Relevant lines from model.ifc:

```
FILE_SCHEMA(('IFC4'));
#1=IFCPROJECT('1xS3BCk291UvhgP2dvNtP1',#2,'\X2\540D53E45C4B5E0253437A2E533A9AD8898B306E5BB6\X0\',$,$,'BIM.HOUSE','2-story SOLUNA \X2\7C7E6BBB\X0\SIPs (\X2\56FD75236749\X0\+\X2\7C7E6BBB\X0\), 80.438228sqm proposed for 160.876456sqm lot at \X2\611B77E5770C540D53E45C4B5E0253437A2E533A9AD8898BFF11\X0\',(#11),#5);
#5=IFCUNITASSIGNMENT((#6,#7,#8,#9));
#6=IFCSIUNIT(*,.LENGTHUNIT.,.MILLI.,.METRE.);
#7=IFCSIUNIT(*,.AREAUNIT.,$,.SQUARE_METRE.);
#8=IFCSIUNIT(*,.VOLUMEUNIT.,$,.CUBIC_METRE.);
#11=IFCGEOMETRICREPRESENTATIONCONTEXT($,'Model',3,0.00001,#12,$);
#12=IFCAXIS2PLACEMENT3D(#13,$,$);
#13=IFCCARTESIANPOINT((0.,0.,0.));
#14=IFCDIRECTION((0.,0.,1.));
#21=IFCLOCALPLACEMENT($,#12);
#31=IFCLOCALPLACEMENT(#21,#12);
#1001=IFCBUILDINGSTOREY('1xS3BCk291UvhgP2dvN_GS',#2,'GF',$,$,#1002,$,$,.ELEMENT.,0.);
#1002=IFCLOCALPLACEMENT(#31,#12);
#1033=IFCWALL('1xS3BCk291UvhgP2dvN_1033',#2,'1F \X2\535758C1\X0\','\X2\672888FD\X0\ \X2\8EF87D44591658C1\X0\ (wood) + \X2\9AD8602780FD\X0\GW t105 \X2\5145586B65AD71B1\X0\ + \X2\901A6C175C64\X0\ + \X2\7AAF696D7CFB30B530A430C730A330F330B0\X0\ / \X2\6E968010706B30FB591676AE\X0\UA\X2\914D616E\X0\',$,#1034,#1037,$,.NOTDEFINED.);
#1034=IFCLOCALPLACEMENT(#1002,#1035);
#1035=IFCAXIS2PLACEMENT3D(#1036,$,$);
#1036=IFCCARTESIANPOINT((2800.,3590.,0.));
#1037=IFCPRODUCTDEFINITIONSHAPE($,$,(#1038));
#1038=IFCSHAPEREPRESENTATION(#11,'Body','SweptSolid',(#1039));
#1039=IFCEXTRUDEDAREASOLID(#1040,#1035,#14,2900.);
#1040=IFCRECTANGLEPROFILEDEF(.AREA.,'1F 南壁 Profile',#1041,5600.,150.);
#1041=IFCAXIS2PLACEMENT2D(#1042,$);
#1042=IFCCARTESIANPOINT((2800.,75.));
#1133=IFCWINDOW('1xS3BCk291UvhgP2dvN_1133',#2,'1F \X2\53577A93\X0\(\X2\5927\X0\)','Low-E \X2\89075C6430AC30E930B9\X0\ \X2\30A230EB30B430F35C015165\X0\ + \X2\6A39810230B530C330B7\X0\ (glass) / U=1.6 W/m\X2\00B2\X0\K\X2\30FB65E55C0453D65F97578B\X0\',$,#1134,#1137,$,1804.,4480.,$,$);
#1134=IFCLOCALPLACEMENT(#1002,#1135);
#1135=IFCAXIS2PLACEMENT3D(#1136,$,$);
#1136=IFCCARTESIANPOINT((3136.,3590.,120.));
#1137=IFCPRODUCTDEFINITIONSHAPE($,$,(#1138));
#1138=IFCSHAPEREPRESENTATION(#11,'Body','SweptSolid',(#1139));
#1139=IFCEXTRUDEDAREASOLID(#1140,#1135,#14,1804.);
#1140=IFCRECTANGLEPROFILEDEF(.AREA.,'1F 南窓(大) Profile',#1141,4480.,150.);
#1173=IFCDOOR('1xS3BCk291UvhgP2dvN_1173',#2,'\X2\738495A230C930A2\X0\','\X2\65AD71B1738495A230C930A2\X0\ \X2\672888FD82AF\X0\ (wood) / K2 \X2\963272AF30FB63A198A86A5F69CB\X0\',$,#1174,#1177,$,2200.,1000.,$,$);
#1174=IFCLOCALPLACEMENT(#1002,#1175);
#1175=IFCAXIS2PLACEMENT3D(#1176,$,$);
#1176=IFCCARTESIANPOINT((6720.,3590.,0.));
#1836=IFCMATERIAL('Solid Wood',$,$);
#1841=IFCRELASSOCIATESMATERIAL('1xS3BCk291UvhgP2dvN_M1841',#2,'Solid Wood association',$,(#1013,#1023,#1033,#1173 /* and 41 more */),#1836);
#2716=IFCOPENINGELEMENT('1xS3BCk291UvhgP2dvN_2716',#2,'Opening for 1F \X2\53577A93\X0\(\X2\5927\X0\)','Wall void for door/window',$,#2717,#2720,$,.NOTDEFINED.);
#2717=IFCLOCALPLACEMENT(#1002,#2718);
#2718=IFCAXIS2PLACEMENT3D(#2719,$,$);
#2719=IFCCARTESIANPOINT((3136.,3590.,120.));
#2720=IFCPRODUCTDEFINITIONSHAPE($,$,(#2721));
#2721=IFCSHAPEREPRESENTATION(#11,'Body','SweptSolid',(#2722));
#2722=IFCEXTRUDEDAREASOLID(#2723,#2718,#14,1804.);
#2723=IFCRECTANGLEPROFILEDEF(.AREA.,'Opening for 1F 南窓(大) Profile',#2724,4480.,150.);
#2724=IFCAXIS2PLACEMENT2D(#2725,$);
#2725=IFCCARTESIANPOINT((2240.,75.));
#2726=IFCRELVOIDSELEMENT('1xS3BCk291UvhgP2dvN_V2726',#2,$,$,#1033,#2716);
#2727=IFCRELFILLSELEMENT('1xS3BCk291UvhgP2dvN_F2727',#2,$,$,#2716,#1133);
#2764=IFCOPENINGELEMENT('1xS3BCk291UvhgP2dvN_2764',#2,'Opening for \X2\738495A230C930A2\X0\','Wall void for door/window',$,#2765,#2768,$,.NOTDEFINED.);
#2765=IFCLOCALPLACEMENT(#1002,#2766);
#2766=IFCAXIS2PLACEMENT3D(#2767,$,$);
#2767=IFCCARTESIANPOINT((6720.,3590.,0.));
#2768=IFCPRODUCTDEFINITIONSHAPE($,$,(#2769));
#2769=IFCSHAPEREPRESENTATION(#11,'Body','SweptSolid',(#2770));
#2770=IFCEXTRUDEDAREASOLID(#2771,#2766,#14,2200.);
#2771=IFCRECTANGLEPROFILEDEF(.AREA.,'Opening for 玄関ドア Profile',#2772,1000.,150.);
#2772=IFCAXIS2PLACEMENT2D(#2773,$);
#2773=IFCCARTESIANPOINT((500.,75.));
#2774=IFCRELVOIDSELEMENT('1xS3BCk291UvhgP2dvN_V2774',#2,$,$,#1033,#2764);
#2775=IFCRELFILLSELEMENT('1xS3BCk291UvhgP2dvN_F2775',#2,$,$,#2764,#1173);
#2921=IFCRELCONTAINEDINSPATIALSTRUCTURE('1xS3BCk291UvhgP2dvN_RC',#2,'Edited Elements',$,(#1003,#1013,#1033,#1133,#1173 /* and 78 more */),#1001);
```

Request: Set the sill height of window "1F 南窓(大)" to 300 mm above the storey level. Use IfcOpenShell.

```python
import numpy as np
import ifcopenshell
import ifcopenshell.api.geometry
import ifcopenshell.geom
import ifcopenshell.util.element
import ifcopenshell.util.placement
import ifcopenshell.util.shape
import ifcopenshell.util.unit

model = ifcopenshell.open("model.ifc")
unit_scale = ifcopenshell.util.unit.calculate_unit_scale(model)

window = model.by_guid("1xS3BCk291UvhgP2dvN_1133")
opening = window.FillsVoids[0].RelatingOpeningElement
storey = ifcopenshell.util.element.get_container(window, ifc_class="IfcBuildingStorey")
level = ifcopenshell.util.placement.get_local_placement(storey.ObjectPlacement)[2, 3]

# The opening's origin need not be at the sill, so measure its lowest point.
shape = ifcopenshell.geom.create_shape(ifcopenshell.geom.settings(), opening)
bottom = ifcopenshell.util.shape.get_shape_bottom_elevation(shape, shape.geometry) / unit_scale
dz = level + 0.3 / unit_scale - bottom

shift = np.array([0.0, 0.0, dz])
# The window is not placed relative to its opening, so move both.
for product in (opening, window):
    matrix = ifcopenshell.util.placement.get_local_placement(product.ObjectPlacement)
    matrix[:3, 3] += shift
    ifcopenshell.api.geometry.edit_object_placement(model, product=product, matrix=matrix, is_si=False)

print(f"moved by {dz * unit_scale:+.3f} m")

model.write("model-out.ifc")
```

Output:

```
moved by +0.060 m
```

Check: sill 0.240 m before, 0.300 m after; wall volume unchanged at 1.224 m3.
